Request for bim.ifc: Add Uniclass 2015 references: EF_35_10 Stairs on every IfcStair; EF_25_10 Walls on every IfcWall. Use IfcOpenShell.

First a look at what the model holds.

```python
import ifcopenshell

model = ifcopenshell.open("bim.ifc")
print(model.schema)
print("classifications:", [c.Name for c in model.by_type("IfcClassification")])
for ifc_class in ("IfcDoor", "IfcRoof", "IfcStair", "IfcWall", "IfcWindow"):
    print(ifc_class, len(model.by_type(ifc_class)))
```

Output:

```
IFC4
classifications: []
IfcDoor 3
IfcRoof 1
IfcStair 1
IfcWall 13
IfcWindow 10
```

```python
import ifcopenshell
import ifcopenshell.api.classification

model = ifcopenshell.open("bim.ifc")

system = ifcopenshell.api.classification.add_classification(model, classification="Uniclass 2015")

codes = {
    "IfcStair": ("EF_35_10", "Stairs"),
    "IfcWall": ("EF_25_10", "Walls"),
}
for ifc_class, (code, name) in codes.items():
    products = model.by_type(ifc_class)
    ifcopenshell.api.classification.add_reference(
        model, products=products, classification=system, identification=code, name=name
    )
    print(code, len(products))

model.write("bim_rev.ifc")
```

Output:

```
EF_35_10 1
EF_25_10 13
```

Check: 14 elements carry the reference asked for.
